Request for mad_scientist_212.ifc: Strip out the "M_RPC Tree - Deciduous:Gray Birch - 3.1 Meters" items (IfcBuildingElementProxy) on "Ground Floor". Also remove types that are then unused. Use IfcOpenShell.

First a look at what the model holds.

```python
import ifcopenshell
import ifcopenshell.util.element

model = ifcopenshell.open("mad_scientist_212.ifc")
print(model.schema)
storey = next(s for s in model.by_type("IfcBuildingStorey") if s.Name == "Ground Floor")
proxies = [e for e in ifcopenshell.util.element.get_decomposition(storey) if e.is_a("IfcBuildingElementProxy")]
seen = {}
for e in proxies:
    element_type = ifcopenshell.util.element.get_type(e)
    name = element_type.Name if element_type not in (None, e) else None
    seen[name] = seen.get(name, 0) + 1
for name, count in sorted(seen.items(), key=str):
    print(count, "x", name)
```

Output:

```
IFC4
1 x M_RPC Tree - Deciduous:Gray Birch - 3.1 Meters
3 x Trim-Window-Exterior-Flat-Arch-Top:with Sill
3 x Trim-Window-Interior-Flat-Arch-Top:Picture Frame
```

```python
import ifcopenshell
import ifcopenshell.api.root
import ifcopenshell.util.element

model = ifcopenshell.open("mad_scientist_212.ifc")

storey = next(s for s in model.by_type("IfcBuildingStorey") if s.Name == "Ground Floor")
proxies = [e for e in ifcopenshell.util.element.get_decomposition(storey) if e.is_a("IfcBuildingElementProxy")]
targets = [e for e in proxies if (t := ifcopenshell.util.element.get_type(e)) not in (None, e) and t.Name == "M_RPC Tree - Deciduous:Gray Birch - 3.1 Meters"]
types = {ifcopenshell.util.element.get_type(e) for e in targets} - {None, *targets}

for e in targets:
    ifcopenshell.api.root.remove_product(model, product=e)
print(len(targets), "removed")

unused = [t for t in types if not ifcopenshell.util.element.get_types(t)]
for t in unused:
    ifcopenshell.api.root.remove_product(model, product=t)
print(len(unused), "unused types removed")

model.write("mad_scientist_212_edited.ifc")
```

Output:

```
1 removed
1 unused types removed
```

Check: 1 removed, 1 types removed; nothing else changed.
